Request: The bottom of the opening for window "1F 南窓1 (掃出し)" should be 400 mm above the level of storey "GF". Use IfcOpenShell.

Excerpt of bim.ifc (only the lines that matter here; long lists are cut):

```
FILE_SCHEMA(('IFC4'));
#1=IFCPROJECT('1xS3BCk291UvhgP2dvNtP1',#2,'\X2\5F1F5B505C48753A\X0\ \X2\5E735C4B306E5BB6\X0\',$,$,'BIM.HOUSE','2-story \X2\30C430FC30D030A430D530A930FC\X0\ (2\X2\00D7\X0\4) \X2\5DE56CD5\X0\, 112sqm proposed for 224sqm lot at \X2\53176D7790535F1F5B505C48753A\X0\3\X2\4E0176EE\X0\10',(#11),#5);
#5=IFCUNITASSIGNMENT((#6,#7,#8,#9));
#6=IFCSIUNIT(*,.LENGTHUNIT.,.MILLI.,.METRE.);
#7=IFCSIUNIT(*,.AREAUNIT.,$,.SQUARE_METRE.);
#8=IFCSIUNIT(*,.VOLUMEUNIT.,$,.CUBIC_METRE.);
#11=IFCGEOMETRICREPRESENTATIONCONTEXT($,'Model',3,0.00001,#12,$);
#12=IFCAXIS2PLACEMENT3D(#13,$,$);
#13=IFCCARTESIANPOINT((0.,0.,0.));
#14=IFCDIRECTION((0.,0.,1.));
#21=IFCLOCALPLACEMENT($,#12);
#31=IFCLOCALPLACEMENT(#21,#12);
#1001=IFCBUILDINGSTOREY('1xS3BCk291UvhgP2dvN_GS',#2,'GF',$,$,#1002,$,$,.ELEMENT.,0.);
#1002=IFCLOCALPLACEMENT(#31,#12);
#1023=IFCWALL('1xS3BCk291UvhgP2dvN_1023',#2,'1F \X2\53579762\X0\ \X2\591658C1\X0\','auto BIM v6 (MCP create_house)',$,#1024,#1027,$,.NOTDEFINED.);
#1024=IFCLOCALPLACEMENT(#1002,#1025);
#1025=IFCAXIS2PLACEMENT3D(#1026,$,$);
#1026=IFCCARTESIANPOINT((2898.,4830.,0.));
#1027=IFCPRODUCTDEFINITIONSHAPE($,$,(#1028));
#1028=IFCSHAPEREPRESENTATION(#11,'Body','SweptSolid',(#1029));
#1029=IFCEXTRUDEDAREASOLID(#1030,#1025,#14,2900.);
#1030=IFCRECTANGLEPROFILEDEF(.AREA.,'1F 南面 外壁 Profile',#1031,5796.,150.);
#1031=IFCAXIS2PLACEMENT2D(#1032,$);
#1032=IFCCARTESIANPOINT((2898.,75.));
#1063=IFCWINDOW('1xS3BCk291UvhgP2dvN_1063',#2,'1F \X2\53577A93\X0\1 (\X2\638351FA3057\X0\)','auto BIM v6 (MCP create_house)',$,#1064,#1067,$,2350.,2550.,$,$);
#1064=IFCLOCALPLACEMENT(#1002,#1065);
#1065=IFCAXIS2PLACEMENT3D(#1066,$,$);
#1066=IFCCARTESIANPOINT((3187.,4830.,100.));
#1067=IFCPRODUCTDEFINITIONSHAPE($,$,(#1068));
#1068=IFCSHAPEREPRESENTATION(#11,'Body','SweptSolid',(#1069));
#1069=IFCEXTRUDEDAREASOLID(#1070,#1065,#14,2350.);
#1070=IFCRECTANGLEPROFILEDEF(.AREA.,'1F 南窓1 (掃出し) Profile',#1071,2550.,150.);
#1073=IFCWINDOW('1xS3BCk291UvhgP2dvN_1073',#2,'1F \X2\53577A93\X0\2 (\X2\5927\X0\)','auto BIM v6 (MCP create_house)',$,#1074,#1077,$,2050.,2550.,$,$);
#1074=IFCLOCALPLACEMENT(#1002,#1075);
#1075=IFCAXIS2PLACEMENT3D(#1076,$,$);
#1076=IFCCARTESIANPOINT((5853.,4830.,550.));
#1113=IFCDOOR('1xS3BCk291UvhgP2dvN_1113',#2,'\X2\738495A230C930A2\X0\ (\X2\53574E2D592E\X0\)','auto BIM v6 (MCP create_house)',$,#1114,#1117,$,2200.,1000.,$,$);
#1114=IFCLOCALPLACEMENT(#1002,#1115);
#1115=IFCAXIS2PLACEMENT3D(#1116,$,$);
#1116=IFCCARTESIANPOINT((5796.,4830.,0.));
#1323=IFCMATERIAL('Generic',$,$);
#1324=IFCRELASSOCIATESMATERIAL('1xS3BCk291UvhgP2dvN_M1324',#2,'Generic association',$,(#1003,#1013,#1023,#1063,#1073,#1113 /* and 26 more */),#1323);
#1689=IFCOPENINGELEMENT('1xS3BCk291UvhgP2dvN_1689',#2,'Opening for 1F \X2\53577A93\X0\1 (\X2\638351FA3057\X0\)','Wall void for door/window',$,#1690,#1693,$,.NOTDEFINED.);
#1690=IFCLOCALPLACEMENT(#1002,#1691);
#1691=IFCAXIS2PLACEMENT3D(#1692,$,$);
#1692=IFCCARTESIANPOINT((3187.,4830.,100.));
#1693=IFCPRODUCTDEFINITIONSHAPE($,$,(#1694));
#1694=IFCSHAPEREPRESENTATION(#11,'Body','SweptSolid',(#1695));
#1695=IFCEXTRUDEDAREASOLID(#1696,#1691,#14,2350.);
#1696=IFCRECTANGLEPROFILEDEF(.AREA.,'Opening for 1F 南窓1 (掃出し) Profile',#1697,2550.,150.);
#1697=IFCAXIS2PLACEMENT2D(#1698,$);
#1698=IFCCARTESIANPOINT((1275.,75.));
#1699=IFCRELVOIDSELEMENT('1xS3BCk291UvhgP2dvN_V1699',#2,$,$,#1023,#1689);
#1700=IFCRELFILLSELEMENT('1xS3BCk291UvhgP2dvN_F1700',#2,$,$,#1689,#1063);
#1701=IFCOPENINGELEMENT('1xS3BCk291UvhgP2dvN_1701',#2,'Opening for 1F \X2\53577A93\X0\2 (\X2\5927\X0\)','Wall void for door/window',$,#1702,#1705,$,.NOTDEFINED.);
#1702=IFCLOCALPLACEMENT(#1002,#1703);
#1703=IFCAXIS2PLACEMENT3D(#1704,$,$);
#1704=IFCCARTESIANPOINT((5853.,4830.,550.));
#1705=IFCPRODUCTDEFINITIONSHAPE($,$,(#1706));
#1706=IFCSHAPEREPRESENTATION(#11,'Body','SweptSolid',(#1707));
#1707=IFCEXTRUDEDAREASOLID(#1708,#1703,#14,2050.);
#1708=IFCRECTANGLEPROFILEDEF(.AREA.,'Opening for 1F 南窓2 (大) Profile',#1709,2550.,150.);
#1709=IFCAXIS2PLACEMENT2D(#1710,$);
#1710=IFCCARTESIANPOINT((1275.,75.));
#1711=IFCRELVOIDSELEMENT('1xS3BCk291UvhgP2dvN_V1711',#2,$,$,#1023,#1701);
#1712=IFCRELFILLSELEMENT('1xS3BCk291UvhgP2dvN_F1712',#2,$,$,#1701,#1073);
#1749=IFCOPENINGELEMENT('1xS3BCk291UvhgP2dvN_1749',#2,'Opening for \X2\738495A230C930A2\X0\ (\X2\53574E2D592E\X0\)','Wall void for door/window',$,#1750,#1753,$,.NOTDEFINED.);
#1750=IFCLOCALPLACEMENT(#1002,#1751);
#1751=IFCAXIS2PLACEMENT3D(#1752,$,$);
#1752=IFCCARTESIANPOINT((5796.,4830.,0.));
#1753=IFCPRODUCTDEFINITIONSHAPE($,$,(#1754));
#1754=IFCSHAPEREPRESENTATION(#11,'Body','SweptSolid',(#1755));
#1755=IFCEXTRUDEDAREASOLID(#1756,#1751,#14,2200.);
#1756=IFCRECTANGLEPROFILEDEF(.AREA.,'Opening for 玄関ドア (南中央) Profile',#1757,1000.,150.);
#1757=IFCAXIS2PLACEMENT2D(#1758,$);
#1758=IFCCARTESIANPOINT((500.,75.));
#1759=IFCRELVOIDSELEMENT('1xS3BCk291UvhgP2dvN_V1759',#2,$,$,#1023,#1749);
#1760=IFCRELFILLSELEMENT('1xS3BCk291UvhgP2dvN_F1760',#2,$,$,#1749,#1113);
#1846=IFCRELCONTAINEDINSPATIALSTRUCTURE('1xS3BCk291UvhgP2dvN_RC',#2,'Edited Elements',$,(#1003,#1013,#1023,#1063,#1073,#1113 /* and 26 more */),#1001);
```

```python
import numpy as np
import ifcopenshell
import ifcopenshell.api.geometry
import ifcopenshell.geom
import ifcopenshell.util.element
import ifcopenshell.util.placement
import ifcopenshell.util.shape
import ifcopenshell.util.unit

model = ifcopenshell.open("bim.ifc")
unit_scale = ifcopenshell.util.unit.calculate_unit_scale(model)

window = model.by_id(1063)
opening = window.FillsVoids[0].RelatingOpeningElement
storey = ifcopenshell.util.element.get_container(window, ifc_class="IfcBuildingStorey")
level = ifcopenshell.util.placement.get_local_placement(storey.ObjectPlacement)[2, 3]

# The opening's origin need not be at the sill, so measure its lowest point.
shape = ifcopenshell.geom.create_shape(ifcopenshell.geom.settings(), opening)
bottom = ifcopenshell.util.shape.get_shape_bottom_elevation(shape, shape.geometry) / unit_scale
dz = level + 400.0 - bottom

shift = np.array([0.0, 0.0, dz])
# The window is not placed relative to its opening, so move both.
for product in (opening, window):
    matrix = ifcopenshell.util.placement.get_local_placement(product.ObjectPlacement)
    matrix[:3, 3] += shift
    ifcopenshell.api.geometry.edit_object_placement(model, product=product, matrix=matrix, is_si=False)

print(f"moved by {dz * unit_scale:+.3f} m")

model.write("bim_rev.ifc")
```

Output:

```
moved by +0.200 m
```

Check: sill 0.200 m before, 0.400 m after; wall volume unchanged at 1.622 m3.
